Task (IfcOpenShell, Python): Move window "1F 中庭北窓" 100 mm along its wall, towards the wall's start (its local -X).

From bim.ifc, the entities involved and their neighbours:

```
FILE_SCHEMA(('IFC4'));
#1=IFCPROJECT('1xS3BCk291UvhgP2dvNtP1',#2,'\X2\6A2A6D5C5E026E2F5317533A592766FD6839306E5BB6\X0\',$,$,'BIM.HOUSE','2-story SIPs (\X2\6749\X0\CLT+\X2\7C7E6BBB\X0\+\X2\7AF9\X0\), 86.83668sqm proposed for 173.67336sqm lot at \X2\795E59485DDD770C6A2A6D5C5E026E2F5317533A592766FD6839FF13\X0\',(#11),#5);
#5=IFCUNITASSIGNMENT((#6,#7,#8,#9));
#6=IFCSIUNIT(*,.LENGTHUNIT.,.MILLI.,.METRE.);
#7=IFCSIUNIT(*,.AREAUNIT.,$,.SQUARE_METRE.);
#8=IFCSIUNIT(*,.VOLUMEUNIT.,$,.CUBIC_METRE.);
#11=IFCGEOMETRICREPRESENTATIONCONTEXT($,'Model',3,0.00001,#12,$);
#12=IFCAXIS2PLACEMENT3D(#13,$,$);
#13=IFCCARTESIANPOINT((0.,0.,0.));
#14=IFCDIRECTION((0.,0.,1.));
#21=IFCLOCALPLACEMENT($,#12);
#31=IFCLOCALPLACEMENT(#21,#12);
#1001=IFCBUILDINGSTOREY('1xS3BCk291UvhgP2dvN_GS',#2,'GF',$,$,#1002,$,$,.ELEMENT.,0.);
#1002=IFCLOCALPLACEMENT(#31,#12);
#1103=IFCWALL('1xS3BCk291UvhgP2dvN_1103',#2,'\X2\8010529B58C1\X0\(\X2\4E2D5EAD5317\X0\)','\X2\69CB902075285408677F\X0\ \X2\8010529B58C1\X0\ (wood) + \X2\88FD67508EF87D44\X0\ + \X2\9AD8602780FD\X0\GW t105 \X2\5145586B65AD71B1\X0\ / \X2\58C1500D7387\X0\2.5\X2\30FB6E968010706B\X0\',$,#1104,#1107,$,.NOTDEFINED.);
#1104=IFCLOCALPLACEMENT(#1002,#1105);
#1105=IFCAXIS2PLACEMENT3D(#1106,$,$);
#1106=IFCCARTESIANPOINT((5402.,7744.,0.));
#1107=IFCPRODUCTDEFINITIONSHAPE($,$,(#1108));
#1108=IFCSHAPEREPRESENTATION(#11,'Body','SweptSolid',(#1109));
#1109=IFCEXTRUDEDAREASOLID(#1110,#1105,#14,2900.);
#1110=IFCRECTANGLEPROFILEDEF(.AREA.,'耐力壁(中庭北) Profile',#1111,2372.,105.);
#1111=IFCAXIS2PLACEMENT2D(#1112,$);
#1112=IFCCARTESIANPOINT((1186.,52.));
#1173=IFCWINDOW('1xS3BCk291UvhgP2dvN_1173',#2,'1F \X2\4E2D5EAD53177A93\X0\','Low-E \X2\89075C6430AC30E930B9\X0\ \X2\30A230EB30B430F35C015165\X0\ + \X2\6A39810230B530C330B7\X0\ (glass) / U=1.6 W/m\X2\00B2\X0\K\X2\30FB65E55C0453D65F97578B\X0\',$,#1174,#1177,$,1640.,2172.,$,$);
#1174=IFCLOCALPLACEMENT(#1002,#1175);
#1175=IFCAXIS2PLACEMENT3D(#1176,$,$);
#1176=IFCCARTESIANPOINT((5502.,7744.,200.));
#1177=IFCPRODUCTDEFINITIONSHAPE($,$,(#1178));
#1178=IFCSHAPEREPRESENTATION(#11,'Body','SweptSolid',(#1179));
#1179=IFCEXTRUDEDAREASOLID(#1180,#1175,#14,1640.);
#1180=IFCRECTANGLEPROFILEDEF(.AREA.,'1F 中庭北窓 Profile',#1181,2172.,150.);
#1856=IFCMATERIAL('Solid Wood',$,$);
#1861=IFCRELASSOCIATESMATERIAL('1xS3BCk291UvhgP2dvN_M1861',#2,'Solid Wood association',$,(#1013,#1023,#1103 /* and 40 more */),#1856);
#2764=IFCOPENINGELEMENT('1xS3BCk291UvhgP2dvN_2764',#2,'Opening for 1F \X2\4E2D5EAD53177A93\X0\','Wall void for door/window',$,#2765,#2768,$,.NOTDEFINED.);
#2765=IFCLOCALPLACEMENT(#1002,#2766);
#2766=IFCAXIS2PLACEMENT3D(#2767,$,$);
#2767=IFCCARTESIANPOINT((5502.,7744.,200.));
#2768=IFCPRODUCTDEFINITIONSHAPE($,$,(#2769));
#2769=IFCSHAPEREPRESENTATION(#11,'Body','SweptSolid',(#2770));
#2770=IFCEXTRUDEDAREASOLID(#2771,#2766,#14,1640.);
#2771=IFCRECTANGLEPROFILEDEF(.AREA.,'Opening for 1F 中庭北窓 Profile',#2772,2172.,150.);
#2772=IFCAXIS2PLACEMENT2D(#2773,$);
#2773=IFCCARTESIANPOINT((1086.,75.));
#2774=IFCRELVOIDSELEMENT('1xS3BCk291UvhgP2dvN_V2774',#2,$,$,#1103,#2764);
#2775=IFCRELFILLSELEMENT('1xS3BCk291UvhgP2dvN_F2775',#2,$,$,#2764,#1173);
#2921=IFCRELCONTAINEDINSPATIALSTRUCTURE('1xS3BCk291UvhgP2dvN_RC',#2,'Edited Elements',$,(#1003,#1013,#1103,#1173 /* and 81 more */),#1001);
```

```python
import ifcopenshell
import ifcopenshell.api.geometry
import ifcopenshell.util.placement
import ifcopenshell.util.unit

model = ifcopenshell.open("bim.ifc")
unit_scale = ifcopenshell.util.unit.calculate_unit_scale(model)

window = model.by_guid("1xS3BCk291UvhgP2dvN_1173")
opening = window.FillsVoids[0].RelatingOpeningElement
wall = opening.VoidsElements[0].RelatingBuildingElement

wall_matrix = ifcopenshell.util.placement.get_local_placement(wall.ObjectPlacement)
shift = wall_matrix[:3, 0] * -0.1 / unit_scale
before = ifcopenshell.util.placement.get_local_placement(window.ObjectPlacement)[:3, 3].copy()

# The window is not placed relative to its opening, so move both.
for product in (opening, window):
    matrix = ifcopenshell.util.placement.get_local_placement(product.ObjectPlacement)
    matrix[:3, 3] += shift
    ifcopenshell.api.geometry.edit_object_placement(model, product=product, matrix=matrix, is_si=False)

after = ifcopenshell.util.placement.get_local_placement(window.ObjectPlacement)[:3, 3]
print("window moved by", (after - before).round(3) + 0.0)

model.write("bim_v2.ifc")
```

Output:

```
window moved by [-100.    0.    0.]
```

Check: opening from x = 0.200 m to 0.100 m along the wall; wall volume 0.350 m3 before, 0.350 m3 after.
